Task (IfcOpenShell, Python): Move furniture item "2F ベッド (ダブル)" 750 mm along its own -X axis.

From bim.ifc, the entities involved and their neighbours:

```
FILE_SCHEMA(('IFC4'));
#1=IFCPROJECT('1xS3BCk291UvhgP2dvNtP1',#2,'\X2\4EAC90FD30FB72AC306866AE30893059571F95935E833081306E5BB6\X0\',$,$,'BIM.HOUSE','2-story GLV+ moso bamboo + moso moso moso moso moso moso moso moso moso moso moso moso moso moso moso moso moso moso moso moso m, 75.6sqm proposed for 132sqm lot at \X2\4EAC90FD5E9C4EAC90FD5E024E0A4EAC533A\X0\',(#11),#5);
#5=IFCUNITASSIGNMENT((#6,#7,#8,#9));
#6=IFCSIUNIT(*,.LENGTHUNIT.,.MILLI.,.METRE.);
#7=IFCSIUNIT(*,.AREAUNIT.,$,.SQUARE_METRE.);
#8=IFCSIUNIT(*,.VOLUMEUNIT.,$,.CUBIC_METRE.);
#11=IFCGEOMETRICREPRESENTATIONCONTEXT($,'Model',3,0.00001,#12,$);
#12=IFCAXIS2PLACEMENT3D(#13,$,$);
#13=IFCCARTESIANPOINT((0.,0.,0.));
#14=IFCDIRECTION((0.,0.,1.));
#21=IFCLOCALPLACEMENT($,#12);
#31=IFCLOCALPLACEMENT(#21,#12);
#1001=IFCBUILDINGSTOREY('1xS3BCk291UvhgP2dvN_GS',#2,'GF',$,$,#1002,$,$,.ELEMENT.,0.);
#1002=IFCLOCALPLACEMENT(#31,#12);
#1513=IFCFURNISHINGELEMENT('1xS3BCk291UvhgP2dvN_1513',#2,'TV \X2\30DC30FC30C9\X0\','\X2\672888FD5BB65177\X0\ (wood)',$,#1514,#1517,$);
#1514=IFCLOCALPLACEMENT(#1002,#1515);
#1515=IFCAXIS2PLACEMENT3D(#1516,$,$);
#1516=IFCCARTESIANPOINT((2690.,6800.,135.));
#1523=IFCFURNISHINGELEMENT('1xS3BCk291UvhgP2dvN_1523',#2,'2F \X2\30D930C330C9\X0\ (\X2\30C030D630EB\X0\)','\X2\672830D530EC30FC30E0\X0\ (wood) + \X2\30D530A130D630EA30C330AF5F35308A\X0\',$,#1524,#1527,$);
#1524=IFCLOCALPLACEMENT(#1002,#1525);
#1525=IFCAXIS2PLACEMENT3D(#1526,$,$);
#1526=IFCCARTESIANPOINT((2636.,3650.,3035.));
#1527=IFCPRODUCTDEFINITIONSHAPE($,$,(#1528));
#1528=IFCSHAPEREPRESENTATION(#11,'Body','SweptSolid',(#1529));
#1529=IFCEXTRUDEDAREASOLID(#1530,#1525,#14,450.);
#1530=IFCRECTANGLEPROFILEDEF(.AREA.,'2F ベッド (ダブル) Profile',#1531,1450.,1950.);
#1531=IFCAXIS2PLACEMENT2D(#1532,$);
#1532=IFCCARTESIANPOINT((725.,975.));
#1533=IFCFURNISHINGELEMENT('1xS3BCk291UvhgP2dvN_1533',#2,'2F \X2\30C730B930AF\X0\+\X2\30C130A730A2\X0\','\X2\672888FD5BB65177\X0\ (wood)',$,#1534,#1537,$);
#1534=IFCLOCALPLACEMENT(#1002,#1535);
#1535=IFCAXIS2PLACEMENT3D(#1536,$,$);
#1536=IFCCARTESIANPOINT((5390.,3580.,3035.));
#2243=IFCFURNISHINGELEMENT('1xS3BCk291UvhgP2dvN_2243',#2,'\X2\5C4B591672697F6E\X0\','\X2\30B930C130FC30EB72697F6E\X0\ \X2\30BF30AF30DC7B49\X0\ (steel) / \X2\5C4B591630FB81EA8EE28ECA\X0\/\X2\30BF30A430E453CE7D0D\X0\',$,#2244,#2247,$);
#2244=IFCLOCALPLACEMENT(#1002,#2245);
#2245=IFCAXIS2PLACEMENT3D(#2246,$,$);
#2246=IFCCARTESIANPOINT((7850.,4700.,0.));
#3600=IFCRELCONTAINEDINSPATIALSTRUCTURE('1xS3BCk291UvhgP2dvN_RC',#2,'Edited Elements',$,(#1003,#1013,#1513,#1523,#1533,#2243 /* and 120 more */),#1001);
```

```python
import ifcopenshell
import ifcopenshell.api.geometry
import ifcopenshell.util.placement
import ifcopenshell.util.unit

model = ifcopenshell.open("bim.ifc")
unit_scale = ifcopenshell.util.unit.calculate_unit_scale(model)

item = model.by_id(1523)
matrix = ifcopenshell.util.placement.get_local_placement(item.ObjectPlacement)
matrix[:3, 3] -= matrix[:3, 0] * 0.75 / unit_scale
ifcopenshell.api.geometry.edit_object_placement(model, product=item, matrix=matrix, is_si=False)

print(ifcopenshell.util.placement.get_local_placement(item.ObjectPlacement).round(3) + 0.0)

model.write("bim_edited.ifc")
```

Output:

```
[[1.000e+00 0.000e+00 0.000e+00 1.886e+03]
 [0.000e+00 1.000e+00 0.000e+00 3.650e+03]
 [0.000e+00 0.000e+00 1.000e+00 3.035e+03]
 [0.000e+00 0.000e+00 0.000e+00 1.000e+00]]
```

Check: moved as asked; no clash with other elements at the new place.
